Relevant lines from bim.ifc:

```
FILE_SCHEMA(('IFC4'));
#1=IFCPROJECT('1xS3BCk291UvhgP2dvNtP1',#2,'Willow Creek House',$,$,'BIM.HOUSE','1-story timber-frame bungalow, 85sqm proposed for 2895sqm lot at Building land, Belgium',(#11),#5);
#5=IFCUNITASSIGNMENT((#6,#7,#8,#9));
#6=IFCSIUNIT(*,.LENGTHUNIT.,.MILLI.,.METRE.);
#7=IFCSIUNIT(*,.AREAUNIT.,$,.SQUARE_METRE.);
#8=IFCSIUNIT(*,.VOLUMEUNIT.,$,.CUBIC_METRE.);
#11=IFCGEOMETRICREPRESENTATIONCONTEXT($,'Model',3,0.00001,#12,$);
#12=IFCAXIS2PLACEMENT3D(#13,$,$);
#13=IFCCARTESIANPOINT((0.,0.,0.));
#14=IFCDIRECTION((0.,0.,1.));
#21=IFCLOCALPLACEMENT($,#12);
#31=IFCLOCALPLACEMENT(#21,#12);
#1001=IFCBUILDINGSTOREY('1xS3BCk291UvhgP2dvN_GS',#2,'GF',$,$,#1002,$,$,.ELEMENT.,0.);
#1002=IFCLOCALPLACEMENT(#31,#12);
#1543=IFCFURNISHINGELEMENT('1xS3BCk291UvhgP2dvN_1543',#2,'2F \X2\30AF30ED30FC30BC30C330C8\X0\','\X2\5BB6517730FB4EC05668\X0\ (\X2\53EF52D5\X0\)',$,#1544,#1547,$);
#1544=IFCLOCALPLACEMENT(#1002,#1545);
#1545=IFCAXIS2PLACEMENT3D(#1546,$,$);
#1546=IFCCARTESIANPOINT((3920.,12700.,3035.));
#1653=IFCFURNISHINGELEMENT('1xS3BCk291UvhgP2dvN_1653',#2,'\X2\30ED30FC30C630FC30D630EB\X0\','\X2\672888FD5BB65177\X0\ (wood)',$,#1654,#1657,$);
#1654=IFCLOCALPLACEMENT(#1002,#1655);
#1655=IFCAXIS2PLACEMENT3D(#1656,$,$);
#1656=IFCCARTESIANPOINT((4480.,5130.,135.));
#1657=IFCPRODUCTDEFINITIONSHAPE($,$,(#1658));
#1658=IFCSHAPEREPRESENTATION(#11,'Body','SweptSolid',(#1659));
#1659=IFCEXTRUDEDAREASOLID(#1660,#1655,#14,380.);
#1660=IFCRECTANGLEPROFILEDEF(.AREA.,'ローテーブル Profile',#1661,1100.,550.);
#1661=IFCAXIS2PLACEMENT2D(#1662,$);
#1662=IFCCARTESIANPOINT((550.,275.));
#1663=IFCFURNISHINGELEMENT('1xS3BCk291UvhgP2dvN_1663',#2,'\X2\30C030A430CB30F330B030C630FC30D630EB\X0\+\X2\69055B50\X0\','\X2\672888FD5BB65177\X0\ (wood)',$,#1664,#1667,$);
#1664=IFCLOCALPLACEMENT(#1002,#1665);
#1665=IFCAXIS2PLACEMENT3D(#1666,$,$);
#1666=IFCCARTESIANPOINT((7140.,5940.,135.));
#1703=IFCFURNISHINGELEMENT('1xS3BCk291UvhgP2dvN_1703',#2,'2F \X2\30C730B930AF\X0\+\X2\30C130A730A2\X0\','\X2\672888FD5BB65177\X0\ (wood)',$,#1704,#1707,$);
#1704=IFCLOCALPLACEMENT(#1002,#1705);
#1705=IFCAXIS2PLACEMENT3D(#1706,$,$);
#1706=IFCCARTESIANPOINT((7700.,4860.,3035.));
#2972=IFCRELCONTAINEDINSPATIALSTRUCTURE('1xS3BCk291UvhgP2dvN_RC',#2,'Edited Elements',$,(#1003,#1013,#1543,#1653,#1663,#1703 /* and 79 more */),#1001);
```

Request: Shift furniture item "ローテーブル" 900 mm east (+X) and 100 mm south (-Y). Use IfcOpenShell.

```python
import ifcopenshell
import ifcopenshell.api.geometry
import ifcopenshell.util.placement
import ifcopenshell.util.unit

model = ifcopenshell.open("bim.ifc")
unit_scale = ifcopenshell.util.unit.calculate_unit_scale(model)

item = model.by_guid("1xS3BCk291UvhgP2dvN_1653")
matrix = ifcopenshell.util.placement.get_local_placement(item.ObjectPlacement)
matrix[0, 3] += 0.9 / unit_scale
matrix[1, 3] -= 0.1 / unit_scale
ifcopenshell.api.geometry.edit_object_placement(model, product=item, matrix=matrix, is_si=False)

print(ifcopenshell.util.placement.get_local_placement(item.ObjectPlacement).round(3) + 0.0)

model.write("bim-out.ifc")
```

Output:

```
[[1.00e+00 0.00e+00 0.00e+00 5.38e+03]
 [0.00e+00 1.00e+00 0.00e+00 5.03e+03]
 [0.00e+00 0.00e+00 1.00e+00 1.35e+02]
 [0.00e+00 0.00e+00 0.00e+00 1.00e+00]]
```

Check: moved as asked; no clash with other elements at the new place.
